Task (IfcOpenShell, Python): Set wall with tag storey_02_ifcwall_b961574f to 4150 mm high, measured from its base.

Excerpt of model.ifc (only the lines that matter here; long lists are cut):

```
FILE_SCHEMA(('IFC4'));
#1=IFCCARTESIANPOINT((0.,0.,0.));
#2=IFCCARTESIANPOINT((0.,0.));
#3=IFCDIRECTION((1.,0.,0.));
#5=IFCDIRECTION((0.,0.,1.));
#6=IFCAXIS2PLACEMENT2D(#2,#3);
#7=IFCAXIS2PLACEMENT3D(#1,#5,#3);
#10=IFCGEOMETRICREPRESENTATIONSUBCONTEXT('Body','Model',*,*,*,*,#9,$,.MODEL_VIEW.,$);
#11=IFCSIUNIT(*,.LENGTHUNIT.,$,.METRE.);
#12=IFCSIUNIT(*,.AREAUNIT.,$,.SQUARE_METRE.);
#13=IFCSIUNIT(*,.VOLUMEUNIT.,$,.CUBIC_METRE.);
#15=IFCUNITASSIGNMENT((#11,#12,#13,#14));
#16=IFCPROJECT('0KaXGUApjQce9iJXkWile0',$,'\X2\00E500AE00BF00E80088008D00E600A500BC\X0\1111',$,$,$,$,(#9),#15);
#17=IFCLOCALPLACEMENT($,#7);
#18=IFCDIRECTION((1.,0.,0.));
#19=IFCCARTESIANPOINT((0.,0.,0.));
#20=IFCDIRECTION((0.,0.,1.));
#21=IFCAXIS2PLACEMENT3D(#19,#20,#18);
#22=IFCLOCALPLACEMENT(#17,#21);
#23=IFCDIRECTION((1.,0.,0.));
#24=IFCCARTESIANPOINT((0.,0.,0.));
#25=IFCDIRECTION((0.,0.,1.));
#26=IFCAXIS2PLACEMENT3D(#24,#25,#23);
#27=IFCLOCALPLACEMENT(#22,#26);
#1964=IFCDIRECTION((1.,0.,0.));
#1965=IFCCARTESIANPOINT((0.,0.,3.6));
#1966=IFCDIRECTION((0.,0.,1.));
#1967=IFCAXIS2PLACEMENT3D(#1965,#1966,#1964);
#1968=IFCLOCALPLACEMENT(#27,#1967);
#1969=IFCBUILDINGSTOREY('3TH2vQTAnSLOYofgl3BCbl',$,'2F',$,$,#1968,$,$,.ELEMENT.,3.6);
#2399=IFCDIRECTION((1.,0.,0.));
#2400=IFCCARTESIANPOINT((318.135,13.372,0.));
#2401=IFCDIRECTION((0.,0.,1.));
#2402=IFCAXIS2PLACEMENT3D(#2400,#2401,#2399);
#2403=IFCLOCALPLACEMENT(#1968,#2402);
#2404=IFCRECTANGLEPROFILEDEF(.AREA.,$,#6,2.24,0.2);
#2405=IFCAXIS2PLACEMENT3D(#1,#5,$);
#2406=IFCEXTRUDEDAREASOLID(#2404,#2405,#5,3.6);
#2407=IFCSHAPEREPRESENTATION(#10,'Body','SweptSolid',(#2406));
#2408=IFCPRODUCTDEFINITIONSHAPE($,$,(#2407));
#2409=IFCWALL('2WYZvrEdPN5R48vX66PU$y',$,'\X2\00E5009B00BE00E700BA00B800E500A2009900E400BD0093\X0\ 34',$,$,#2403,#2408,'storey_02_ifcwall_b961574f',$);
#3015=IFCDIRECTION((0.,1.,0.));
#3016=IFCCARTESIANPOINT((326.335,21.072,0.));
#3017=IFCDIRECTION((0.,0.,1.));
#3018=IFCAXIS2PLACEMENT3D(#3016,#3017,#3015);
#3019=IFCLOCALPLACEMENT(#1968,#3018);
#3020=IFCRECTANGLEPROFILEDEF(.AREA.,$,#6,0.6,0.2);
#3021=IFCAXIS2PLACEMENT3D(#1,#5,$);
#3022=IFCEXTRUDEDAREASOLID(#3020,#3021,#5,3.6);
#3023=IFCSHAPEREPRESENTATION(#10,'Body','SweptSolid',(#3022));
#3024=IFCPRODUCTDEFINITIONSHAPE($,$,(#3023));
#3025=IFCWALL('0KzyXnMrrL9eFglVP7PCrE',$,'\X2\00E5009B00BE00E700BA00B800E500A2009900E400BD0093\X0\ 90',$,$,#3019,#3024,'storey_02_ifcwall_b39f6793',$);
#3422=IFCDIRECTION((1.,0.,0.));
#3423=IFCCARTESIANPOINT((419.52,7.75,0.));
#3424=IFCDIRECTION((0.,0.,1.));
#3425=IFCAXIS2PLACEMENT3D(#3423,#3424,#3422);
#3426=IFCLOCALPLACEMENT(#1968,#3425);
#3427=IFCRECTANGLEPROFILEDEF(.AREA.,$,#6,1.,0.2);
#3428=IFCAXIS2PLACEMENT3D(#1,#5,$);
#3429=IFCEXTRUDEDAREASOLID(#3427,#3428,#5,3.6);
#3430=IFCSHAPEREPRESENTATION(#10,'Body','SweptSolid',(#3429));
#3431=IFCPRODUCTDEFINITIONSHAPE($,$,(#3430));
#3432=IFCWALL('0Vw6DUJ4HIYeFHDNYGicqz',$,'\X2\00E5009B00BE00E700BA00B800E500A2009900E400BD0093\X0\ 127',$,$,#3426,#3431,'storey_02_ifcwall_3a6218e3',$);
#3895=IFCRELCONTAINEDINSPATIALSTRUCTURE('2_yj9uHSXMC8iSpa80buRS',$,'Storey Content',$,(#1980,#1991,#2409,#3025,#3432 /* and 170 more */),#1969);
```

```python
import ifcopenshell
import ifcopenshell.geom
import ifcopenshell.util.representation
import ifcopenshell.util.shape
import ifcopenshell.util.unit

model = ifcopenshell.open("model.ifc")
unit_scale = ifcopenshell.util.unit.calculate_unit_scale(model)
settings = ifcopenshell.geom.settings()


def volume(element):
    """Net volume in cubic metres, openings subtracted."""
    shape = ifcopenshell.geom.create_shape(settings, element)
    return ifcopenshell.util.shape.get_volume(shape.geometry)


wall = model.by_guid("2WYZvrEdPN5R48vX66PU$y")
before = volume(wall)

body = ifcopenshell.util.representation.get_representation(wall, "Model", "Body")
solid = body.Items[0]
old_height = solid.Depth
solid.Depth = 4.15 / unit_scale
after = volume(wall)

print(f"height {old_height:g} -> {solid.Depth:g}, volume {before:.3f} -> {after:.3f} m3")

model.write("model_rev.ifc")
```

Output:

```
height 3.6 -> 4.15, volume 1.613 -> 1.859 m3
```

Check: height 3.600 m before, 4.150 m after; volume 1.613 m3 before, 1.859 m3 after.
